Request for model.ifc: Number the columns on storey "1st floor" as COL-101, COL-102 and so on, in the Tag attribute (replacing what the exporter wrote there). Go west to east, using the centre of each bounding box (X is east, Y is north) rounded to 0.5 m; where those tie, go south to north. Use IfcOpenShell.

First a look at what the model holds.

```python
import ifcopenshell
import ifcopenshell.util.element
import ifcopenshell.util.placement

model = ifcopenshell.open("model.ifc")
print(model.schema)
storey = next(s for s in model.by_type("IfcBuildingStorey") if s.Name == "1st floor")
columns = [e for e in ifcopenshell.util.element.get_decomposition(storey) if e.is_a("IfcColumn")]
for e in sorted(columns, key=lambda e: e.id()):
    origin = ifcopenshell.util.placement.get_local_placement(e.ObjectPlacement)[:3, 3]
    print(e.id(), e.Tag, e.Name, origin.round(2) + 0.0, sep=" | ")
```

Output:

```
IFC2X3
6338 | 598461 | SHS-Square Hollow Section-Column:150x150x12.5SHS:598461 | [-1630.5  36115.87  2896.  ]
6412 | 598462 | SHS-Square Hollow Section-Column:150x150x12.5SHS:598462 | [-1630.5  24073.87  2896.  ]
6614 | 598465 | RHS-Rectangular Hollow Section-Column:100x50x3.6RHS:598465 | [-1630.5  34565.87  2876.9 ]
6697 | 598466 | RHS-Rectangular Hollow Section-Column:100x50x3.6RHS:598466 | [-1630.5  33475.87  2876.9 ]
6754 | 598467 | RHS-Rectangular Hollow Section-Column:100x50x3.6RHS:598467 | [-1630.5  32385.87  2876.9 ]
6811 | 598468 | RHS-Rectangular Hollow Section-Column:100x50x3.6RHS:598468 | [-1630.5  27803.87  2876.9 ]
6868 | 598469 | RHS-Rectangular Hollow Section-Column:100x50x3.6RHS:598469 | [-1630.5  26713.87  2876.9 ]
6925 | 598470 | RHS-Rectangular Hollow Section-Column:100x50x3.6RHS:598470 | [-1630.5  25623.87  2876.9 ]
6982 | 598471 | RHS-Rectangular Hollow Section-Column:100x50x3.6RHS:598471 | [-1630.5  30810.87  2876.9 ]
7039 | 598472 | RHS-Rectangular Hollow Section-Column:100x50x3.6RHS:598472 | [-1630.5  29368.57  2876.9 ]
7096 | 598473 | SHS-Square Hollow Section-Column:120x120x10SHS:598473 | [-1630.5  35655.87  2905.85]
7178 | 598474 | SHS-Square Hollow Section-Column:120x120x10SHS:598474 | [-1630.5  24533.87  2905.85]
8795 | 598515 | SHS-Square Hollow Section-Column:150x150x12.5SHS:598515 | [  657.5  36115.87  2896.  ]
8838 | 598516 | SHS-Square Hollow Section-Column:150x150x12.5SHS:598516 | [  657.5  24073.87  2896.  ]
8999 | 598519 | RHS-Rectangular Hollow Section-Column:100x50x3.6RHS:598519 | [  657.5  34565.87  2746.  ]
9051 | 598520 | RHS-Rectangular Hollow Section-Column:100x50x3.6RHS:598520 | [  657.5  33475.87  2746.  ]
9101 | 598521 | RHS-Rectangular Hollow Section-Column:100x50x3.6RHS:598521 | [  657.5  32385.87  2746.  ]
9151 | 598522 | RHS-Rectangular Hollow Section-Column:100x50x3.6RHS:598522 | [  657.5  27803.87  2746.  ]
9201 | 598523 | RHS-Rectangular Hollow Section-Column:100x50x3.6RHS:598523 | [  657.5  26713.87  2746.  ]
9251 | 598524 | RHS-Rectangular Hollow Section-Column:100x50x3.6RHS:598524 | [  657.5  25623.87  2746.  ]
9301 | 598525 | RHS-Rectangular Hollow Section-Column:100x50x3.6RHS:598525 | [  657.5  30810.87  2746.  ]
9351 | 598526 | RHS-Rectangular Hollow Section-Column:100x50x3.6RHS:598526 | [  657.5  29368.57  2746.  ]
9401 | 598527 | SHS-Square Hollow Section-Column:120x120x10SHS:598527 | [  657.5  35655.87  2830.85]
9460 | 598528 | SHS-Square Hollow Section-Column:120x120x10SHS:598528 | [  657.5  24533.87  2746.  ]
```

```python
import ifcopenshell
import ifcopenshell.geom
import ifcopenshell.util.element
import ifcopenshell.util.shape

model = ifcopenshell.open("model.ifc")
settings = ifcopenshell.geom.settings()
settings.set("use-world-coords", True)


def centre(element):
    shape = ifcopenshell.geom.create_shape(settings, element)
    return ifcopenshell.util.shape.get_bbox_centroid(shape.geometry)


storey = next(s for s in model.by_type("IfcBuildingStorey") if s.Name == "1st floor")
columns = [e for e in ifcopenshell.util.element.get_decomposition(storey) if e.is_a("IfcColumn")]

# Insertion points can sit at a corner or the storey origin, so sort by the geometry (in metres).
centres = {e: centre(e) for e in columns}
columns.sort(key=lambda e: (round(centres[e][0] / 0.5), centres[e][1]))

for i, e in enumerate(columns, start=1):
    number = f"COL-1{i:02d}"
    e.Tag = number
    print(e.id(), number)

model.write("model_v2.ifc")
```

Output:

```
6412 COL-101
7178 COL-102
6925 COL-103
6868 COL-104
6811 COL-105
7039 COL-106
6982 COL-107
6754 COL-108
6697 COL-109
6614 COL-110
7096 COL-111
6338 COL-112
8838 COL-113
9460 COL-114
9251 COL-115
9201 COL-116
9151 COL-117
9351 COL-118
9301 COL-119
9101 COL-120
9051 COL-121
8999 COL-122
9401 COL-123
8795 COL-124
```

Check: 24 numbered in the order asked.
